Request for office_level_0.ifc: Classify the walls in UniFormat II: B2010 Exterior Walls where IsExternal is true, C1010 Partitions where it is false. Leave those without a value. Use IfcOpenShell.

First a look at what the model holds.

```python
import ifcopenshell
import ifcopenshell.util.element

model = ifcopenshell.open("office_level_0.ifc")
print(model.schema)
print("classifications:", [c.Name for c in model.by_type("IfcClassification")])
values = [ifcopenshell.util.element.get_pset(e, "Pset_WallCommon", "IsExternal") for e in model.by_type("IfcWall")]
for value in (True, False, None):
    print("IsExternal", value, values.count(value))
```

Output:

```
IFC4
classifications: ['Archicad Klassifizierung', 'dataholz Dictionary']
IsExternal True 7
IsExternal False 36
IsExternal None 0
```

```python
import ifcopenshell
import ifcopenshell.api.classification
import ifcopenshell.util.element

model = ifcopenshell.open("office_level_0.ifc")

system = ifcopenshell.api.classification.add_classification(model, classification="UniFormat II")

walls = model.by_type("IfcWall")
external = {e: ifcopenshell.util.element.get_pset(e, "Pset_WallCommon", "IsExternal") for e in walls}
for flag, code, name in ((True, "B2010", "Exterior Walls"), (False, "C1010", "Partitions")):
    products = [e for e in walls if external[e] is flag]
    ifcopenshell.api.classification.add_reference(
        model, products=products, classification=system, identification=code, name=name
    )
    print(code, len(products))

model.write("office_level_0_updated.ifc")
```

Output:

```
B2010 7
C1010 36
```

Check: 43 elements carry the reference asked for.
